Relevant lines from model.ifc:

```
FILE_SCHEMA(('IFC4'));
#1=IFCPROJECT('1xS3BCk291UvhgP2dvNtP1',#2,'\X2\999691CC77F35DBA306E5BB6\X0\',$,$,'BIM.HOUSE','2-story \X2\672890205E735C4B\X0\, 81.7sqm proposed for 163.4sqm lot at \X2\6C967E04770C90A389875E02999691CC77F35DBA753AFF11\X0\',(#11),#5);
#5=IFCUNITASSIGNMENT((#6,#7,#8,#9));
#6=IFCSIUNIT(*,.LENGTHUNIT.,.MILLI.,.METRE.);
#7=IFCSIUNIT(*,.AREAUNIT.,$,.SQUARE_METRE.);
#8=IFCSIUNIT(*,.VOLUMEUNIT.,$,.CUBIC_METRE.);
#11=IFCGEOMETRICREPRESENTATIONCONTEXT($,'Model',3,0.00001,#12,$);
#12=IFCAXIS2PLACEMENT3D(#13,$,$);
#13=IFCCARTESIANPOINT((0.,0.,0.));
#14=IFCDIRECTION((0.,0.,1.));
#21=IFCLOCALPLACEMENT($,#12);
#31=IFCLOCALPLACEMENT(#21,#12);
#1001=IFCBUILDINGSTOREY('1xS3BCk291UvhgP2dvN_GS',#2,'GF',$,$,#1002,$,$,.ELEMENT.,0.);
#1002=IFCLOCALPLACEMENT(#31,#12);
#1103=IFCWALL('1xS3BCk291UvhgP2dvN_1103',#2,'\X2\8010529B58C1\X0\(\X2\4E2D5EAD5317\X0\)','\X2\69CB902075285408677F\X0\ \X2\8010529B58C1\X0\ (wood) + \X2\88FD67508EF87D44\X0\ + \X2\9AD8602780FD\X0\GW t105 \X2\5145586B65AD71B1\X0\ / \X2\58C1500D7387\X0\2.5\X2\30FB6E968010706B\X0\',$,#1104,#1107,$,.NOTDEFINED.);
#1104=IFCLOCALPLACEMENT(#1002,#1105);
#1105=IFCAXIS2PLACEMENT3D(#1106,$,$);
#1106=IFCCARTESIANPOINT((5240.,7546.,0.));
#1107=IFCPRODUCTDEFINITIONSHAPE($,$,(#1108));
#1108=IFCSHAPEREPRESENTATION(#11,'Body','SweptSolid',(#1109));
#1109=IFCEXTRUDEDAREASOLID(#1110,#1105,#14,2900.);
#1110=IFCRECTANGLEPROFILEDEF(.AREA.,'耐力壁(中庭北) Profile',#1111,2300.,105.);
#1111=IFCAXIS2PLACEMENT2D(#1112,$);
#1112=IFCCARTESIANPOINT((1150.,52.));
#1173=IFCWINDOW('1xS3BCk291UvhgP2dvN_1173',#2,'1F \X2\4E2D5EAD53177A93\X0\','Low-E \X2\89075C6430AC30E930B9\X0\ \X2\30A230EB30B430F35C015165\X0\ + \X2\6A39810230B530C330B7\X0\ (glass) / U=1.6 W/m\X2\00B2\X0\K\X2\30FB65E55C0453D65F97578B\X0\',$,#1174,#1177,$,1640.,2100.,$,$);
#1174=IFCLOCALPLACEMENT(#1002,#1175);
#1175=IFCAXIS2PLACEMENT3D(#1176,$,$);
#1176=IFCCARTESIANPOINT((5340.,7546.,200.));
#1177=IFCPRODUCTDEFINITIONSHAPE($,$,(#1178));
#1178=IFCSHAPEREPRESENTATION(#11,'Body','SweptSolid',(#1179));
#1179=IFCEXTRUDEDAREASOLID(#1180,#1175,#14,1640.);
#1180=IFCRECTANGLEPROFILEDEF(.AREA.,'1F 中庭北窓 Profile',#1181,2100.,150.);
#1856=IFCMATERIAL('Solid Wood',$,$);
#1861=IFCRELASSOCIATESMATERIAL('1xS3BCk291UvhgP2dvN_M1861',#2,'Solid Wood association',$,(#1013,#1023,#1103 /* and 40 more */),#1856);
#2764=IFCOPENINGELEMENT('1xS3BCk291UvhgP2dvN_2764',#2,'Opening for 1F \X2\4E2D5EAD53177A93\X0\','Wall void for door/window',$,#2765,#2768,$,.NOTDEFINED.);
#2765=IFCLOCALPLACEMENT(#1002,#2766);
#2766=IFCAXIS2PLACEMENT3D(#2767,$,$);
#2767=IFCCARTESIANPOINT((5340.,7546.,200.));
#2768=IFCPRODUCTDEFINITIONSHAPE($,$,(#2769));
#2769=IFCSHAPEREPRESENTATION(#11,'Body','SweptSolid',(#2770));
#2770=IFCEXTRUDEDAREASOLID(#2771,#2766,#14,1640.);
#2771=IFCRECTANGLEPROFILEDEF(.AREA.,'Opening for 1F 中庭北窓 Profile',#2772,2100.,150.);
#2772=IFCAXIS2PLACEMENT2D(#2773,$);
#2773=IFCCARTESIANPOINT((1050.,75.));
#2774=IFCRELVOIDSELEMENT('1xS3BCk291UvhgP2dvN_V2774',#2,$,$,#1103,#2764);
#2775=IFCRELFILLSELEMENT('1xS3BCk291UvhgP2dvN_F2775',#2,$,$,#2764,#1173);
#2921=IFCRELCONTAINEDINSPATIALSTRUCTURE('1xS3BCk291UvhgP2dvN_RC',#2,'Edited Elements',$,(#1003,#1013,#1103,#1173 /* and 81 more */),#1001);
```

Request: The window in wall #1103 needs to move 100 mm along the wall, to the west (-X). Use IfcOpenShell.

```python
import ifcopenshell
import ifcopenshell.api.geometry
import ifcopenshell.util.placement
import ifcopenshell.util.unit

model = ifcopenshell.open("model.ifc")
unit_scale = ifcopenshell.util.unit.calculate_unit_scale(model)

window = model.by_guid("1xS3BCk291UvhgP2dvN_1173")
opening = window.FillsVoids[0].RelatingOpeningElement
wall = opening.VoidsElements[0].RelatingBuildingElement

wall_matrix = ifcopenshell.util.placement.get_local_placement(wall.ObjectPlacement)
shift = wall_matrix[:3, 0] * -0.1 / unit_scale
before = ifcopenshell.util.placement.get_local_placement(window.ObjectPlacement)[:3, 3].copy()

# The window is not placed relative to its opening, so move both.
for product in (opening, window):
    matrix = ifcopenshell.util.placement.get_local_placement(product.ObjectPlacement)
    matrix[:3, 3] += shift
    ifcopenshell.api.geometry.edit_object_placement(model, product=product, matrix=matrix, is_si=False)

after = ifcopenshell.util.placement.get_local_placement(window.ObjectPlacement)[:3, 3]
print("window moved by", (after - before).round(3) + 0.0)

model.write("model_rev.ifc")
```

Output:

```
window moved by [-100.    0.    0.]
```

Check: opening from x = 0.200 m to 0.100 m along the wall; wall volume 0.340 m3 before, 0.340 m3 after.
